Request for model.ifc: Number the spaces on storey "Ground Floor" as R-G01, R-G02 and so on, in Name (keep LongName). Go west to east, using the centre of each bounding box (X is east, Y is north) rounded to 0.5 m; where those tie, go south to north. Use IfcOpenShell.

First a look at what the model holds.

```python
import ifcopenshell
import ifcopenshell.util.element
import ifcopenshell.util.placement

model = ifcopenshell.open("model.ifc")
print(model.schema)
storey = next(s for s in model.by_type("IfcBuildingStorey") if s.Name == "Ground Floor")
spaces = [e for e in ifcopenshell.util.element.get_decomposition(storey) if e.is_a("IfcSpace")]
for e in sorted(spaces, key=lambda e: e.id()):
    origin = ifcopenshell.util.placement.get_local_placement(e.ObjectPlacement)[:3, 3]
    print(e.id(), e.Name, e.LongName, origin.round(2) + 0.0, sep=" | ")
```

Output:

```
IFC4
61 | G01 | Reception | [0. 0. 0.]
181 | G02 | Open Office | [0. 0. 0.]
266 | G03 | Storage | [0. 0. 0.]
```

```python
import ifcopenshell
import ifcopenshell.geom
import ifcopenshell.util.element
import ifcopenshell.util.shape

model = ifcopenshell.open("model.ifc")
settings = ifcopenshell.geom.settings()
settings.set("use-world-coords", True)


def centre(element):
    shape = ifcopenshell.geom.create_shape(settings, element)
    return ifcopenshell.util.shape.get_bbox_centroid(shape.geometry)


storey = next(s for s in model.by_type("IfcBuildingStorey") if s.Name == "Ground Floor")
spaces = [e for e in ifcopenshell.util.element.get_decomposition(storey) if e.is_a("IfcSpace")]

# Insertion points can sit at a corner or the storey origin, so sort by the geometry (in metres).
centres = {e: centre(e) for e in spaces}
spaces.sort(key=lambda e: (round(centres[e][0] / 0.5), centres[e][1]))

for i, e in enumerate(spaces, start=1):
    number = f"R-G{i:02d}"
    e.Name = number
    print(e.id(), number)

model.write("model-out.ifc")
```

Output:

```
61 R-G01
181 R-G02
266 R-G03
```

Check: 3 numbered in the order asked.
